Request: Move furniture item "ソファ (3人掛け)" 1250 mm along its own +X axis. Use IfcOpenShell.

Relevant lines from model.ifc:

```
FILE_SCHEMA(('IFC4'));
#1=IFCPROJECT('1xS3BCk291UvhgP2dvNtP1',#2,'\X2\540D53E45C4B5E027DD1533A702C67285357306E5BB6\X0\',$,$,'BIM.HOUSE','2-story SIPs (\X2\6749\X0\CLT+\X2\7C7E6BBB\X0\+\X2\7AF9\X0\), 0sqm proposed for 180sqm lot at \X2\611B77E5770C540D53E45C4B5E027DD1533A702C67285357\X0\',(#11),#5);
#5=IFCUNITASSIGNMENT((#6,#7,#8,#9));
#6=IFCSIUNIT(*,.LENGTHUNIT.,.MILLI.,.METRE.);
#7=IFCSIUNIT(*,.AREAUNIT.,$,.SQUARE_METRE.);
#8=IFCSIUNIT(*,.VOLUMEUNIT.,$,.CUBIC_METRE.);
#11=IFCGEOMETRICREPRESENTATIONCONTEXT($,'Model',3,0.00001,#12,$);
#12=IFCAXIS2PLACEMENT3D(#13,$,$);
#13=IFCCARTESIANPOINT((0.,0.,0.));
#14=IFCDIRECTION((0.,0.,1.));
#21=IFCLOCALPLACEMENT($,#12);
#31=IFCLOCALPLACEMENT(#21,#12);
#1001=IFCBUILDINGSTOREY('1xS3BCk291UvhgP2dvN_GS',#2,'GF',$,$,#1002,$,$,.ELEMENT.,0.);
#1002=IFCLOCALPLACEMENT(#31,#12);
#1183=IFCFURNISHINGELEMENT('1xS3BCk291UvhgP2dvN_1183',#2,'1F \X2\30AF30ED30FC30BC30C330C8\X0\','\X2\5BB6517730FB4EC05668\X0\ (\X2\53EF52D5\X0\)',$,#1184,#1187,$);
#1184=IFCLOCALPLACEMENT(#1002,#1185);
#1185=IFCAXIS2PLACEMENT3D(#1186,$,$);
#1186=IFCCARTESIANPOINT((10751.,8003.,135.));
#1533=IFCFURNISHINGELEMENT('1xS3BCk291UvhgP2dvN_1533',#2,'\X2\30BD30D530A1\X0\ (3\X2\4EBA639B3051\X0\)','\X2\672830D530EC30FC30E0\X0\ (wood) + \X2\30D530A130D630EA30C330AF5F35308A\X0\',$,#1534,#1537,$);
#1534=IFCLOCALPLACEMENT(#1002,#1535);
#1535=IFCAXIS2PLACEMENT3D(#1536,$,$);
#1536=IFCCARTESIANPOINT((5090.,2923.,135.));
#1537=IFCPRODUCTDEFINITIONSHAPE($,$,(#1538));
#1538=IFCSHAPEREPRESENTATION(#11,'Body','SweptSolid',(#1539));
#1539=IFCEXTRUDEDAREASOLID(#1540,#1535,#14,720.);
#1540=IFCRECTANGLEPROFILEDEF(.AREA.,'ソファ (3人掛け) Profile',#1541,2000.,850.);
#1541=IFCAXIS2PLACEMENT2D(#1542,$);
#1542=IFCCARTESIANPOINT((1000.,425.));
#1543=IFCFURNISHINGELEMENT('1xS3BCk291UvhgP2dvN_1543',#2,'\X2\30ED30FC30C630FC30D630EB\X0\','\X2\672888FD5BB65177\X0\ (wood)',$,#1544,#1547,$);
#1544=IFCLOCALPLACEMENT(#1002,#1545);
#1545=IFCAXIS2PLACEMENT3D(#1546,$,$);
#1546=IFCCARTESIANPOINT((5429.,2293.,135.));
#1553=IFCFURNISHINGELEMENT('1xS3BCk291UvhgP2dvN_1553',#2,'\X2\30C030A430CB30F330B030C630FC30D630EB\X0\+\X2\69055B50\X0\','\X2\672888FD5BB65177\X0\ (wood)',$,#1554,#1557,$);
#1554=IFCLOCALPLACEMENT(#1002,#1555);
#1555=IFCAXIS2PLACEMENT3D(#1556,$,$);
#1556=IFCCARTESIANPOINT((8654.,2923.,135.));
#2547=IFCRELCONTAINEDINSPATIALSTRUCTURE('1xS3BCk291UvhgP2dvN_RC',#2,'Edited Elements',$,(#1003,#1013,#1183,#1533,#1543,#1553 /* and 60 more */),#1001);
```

```python
import ifcopenshell
import ifcopenshell.api.geometry
import ifcopenshell.util.placement
import ifcopenshell.util.unit

model = ifcopenshell.open("model.ifc")
unit_scale = ifcopenshell.util.unit.calculate_unit_scale(model)

item = model.by_guid("1xS3BCk291UvhgP2dvN_1533")
matrix = ifcopenshell.util.placement.get_local_placement(item.ObjectPlacement)
matrix[:3, 3] += matrix[:3, 0] * 1.25 / unit_scale
ifcopenshell.api.geometry.edit_object_placement(model, product=item, matrix=matrix, is_si=False)

print(ifcopenshell.util.placement.get_local_placement(item.ObjectPlacement).round(3) + 0.0)

model.write("model_edited.ifc")
```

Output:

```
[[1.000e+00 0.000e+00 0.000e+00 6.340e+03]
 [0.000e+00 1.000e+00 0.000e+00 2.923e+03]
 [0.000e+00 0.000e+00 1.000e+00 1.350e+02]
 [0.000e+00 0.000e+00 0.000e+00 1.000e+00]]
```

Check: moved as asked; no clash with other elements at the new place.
